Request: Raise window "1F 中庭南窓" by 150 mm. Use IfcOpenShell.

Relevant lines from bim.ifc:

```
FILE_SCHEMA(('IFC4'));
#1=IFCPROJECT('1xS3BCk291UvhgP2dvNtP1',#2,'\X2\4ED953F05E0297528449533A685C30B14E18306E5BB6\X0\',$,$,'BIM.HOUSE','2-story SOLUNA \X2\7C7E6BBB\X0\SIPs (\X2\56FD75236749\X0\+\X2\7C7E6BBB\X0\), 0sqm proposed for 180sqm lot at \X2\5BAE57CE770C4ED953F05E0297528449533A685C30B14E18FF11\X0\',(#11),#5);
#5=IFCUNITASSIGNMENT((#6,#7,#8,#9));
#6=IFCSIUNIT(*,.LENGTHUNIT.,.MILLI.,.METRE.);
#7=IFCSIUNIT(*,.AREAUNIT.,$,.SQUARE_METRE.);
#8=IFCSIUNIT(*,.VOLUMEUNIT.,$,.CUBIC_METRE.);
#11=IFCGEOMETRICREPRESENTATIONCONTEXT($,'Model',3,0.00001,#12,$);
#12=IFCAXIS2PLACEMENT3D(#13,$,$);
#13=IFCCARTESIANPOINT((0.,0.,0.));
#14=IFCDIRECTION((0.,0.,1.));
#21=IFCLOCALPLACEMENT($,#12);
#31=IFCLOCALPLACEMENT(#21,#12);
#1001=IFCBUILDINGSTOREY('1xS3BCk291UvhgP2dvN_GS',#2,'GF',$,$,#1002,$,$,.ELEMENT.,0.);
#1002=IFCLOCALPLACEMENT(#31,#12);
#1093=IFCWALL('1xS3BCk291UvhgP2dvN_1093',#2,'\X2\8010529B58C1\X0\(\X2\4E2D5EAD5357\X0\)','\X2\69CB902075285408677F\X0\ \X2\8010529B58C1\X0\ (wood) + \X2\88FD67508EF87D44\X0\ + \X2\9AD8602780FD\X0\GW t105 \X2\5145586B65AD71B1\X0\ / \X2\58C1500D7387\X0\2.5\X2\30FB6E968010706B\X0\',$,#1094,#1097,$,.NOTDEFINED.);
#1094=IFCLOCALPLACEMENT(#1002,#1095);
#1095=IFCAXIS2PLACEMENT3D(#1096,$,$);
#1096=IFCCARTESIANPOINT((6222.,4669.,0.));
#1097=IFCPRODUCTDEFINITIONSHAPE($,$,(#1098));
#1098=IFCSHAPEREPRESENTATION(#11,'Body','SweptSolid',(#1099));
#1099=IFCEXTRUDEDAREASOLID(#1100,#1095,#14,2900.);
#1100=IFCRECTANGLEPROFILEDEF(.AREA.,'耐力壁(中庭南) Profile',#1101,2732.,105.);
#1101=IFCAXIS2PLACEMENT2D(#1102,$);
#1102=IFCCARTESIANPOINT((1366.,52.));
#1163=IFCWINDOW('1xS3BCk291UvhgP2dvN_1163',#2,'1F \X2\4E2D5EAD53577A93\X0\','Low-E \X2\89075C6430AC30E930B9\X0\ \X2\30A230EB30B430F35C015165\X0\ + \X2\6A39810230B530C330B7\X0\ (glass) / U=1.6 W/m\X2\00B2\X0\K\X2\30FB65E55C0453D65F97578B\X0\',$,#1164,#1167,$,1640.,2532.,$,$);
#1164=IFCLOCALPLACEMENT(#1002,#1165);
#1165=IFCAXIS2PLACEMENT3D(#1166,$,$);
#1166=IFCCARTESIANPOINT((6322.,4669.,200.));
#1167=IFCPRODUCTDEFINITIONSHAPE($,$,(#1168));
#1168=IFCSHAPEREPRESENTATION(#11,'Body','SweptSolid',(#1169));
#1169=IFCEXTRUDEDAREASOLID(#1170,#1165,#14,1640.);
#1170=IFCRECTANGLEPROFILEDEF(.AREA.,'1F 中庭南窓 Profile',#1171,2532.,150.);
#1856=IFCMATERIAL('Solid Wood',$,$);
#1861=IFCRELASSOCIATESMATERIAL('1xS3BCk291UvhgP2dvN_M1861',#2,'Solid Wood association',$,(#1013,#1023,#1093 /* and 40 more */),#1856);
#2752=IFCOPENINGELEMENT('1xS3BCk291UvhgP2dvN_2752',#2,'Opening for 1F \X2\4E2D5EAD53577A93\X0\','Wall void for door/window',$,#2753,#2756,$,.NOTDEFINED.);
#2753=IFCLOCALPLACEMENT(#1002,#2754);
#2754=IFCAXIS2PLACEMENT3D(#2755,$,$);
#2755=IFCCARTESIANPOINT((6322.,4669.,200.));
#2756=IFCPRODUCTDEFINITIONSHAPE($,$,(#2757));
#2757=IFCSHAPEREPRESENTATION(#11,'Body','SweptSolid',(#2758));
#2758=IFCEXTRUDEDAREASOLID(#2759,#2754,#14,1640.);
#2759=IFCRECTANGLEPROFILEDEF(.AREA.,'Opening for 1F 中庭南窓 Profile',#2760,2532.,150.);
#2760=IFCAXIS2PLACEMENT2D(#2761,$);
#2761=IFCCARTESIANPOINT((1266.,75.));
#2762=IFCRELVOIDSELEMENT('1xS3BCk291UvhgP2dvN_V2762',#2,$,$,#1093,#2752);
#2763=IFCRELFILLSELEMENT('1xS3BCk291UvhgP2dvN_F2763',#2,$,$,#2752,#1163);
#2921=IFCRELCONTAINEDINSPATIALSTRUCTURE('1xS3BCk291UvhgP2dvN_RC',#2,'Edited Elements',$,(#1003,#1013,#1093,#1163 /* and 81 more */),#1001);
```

```python
import numpy as np
import ifcopenshell
import ifcopenshell.api.geometry
import ifcopenshell.util.placement
import ifcopenshell.util.unit

model = ifcopenshell.open("bim.ifc")
unit_scale = ifcopenshell.util.unit.calculate_unit_scale(model)

window = model.by_guid("1xS3BCk291UvhgP2dvN_1163")
opening = window.FillsVoids[0].RelatingOpeningElement
dz = 0.15 / unit_scale

shift = np.array([0.0, 0.0, dz])
# The window is not placed relative to its opening, so move both.
for product in (opening, window):
    matrix = ifcopenshell.util.placement.get_local_placement(product.ObjectPlacement)
    matrix[:3, 3] += shift
    ifcopenshell.api.geometry.edit_object_placement(model, product=product, matrix=matrix, is_si=False)

print(f"moved by {dz * unit_scale:+.3f} m")

model.write("bim_v2.ifc")
```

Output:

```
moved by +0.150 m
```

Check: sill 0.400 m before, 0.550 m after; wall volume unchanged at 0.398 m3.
